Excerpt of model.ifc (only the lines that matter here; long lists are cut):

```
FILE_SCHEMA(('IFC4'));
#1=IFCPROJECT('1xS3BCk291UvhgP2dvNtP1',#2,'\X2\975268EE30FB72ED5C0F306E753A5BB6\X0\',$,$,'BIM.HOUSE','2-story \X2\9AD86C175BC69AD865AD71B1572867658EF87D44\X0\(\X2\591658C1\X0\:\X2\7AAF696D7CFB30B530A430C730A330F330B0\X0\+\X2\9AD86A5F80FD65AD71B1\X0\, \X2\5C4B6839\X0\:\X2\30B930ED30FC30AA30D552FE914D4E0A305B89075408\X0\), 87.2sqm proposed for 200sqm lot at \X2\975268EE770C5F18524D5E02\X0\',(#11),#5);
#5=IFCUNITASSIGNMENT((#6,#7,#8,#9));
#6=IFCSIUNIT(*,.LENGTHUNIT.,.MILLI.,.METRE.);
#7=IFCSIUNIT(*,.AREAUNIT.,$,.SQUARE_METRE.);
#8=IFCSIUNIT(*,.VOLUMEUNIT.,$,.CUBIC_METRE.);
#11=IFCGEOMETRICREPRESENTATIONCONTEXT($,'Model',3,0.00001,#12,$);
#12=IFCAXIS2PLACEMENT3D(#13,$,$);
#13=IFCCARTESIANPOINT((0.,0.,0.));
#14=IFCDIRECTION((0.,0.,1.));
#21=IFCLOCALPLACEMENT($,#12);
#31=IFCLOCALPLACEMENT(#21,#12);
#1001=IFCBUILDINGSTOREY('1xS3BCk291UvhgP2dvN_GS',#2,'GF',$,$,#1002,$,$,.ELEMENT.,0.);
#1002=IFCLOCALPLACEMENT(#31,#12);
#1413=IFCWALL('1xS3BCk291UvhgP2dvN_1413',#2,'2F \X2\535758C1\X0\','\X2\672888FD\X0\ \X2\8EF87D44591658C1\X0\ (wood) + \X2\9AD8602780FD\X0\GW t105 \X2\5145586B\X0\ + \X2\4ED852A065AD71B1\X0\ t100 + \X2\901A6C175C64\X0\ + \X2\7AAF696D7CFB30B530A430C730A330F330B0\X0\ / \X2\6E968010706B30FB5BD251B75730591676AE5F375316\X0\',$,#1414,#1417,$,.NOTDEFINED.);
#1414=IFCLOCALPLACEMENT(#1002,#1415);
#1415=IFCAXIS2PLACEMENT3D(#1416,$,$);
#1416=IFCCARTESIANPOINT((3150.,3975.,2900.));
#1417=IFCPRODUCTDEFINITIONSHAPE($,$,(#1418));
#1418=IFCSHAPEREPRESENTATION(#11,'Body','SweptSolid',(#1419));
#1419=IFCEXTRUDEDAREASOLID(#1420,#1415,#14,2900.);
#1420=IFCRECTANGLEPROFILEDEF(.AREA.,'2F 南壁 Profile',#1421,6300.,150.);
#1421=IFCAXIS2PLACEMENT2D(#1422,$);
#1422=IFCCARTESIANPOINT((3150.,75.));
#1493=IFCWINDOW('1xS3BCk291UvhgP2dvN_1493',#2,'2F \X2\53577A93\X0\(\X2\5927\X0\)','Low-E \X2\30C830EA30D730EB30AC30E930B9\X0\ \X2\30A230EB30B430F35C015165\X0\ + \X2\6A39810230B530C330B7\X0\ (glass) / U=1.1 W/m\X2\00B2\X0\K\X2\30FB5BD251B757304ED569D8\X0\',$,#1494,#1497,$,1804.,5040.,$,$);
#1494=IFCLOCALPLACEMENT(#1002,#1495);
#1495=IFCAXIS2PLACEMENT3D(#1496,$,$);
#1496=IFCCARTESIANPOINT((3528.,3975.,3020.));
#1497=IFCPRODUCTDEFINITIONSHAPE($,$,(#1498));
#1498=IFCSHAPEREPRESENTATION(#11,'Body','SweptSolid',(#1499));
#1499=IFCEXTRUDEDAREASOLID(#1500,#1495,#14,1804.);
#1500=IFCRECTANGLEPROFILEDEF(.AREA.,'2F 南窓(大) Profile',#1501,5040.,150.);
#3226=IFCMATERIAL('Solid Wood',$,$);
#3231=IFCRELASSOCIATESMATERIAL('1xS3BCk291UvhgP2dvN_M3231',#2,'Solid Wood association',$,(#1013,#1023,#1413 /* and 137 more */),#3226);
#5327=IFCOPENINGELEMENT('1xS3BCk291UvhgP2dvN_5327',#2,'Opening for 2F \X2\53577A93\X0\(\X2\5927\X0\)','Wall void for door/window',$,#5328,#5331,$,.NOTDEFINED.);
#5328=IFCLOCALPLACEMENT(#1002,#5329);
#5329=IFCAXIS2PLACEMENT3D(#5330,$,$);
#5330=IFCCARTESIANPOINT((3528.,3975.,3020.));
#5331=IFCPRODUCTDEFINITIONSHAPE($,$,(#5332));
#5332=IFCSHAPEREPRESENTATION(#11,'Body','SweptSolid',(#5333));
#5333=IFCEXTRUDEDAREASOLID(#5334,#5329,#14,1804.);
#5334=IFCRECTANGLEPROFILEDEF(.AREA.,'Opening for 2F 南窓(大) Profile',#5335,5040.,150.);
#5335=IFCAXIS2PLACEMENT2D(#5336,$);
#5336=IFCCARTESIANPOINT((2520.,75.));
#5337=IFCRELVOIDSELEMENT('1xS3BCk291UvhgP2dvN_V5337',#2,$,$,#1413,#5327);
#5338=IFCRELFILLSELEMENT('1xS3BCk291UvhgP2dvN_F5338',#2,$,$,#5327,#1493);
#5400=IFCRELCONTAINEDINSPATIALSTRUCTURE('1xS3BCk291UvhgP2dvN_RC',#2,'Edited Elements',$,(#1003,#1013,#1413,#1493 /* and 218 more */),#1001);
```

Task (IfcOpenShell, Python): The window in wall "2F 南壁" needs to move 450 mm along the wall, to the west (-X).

```python
import ifcopenshell
import ifcopenshell.api.geometry
import ifcopenshell.util.placement

model = ifcopenshell.open("model.ifc")

window = model.by_guid("1xS3BCk291UvhgP2dvN_1493")
opening = window.FillsVoids[0].RelatingOpeningElement
wall = opening.VoidsElements[0].RelatingBuildingElement

wall_matrix = ifcopenshell.util.placement.get_local_placement(wall.ObjectPlacement)
shift = wall_matrix[:3, 0] * -450.0
before = ifcopenshell.util.placement.get_local_placement(window.ObjectPlacement)[:3, 3].copy()

# The window is not placed relative to its opening, so move both.
for product in (opening, window):
    matrix = ifcopenshell.util.placement.get_local_placement(product.ObjectPlacement)
    matrix[:3, 3] += shift
    ifcopenshell.api.geometry.edit_object_placement(model, product=product, matrix=matrix, is_si=False)

after = ifcopenshell.util.placement.get_local_placement(window.ObjectPlacement)[:3, 3]
print("window moved by", (after - before).round(3) + 0.0)

model.write("model_updated.ifc")
```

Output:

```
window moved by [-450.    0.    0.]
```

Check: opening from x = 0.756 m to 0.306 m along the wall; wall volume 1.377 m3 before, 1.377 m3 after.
